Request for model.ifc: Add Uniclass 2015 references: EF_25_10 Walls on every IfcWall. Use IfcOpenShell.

First a look at what the model holds.

```python
import ifcopenshell

model = ifcopenshell.open("model.ifc")
print(model.schema)
print("classifications:", [c.Name for c in model.by_type("IfcClassification")])
for ifc_class in ("IfcDoor", "IfcRoof", "IfcStair", "IfcWall", "IfcWindow"):
    print(ifc_class, len(model.by_type(ifc_class)))
```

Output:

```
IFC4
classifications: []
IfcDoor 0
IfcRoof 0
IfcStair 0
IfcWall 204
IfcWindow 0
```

```python
import ifcopenshell
import ifcopenshell.api.classification

model = ifcopenshell.open("model.ifc")

system = ifcopenshell.api.classification.add_classification(model, classification="Uniclass 2015")

codes = {
    "IfcWall": ("EF_25_10", "Walls"),
}
for ifc_class, (code, name) in codes.items():
    products = model.by_type(ifc_class)
    ifcopenshell.api.classification.add_reference(
        model, products=products, classification=system, identification=code, name=name
    )
    print(code, len(products))

model.write("model_edited.ifc")
```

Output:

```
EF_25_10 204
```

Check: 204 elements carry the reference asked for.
